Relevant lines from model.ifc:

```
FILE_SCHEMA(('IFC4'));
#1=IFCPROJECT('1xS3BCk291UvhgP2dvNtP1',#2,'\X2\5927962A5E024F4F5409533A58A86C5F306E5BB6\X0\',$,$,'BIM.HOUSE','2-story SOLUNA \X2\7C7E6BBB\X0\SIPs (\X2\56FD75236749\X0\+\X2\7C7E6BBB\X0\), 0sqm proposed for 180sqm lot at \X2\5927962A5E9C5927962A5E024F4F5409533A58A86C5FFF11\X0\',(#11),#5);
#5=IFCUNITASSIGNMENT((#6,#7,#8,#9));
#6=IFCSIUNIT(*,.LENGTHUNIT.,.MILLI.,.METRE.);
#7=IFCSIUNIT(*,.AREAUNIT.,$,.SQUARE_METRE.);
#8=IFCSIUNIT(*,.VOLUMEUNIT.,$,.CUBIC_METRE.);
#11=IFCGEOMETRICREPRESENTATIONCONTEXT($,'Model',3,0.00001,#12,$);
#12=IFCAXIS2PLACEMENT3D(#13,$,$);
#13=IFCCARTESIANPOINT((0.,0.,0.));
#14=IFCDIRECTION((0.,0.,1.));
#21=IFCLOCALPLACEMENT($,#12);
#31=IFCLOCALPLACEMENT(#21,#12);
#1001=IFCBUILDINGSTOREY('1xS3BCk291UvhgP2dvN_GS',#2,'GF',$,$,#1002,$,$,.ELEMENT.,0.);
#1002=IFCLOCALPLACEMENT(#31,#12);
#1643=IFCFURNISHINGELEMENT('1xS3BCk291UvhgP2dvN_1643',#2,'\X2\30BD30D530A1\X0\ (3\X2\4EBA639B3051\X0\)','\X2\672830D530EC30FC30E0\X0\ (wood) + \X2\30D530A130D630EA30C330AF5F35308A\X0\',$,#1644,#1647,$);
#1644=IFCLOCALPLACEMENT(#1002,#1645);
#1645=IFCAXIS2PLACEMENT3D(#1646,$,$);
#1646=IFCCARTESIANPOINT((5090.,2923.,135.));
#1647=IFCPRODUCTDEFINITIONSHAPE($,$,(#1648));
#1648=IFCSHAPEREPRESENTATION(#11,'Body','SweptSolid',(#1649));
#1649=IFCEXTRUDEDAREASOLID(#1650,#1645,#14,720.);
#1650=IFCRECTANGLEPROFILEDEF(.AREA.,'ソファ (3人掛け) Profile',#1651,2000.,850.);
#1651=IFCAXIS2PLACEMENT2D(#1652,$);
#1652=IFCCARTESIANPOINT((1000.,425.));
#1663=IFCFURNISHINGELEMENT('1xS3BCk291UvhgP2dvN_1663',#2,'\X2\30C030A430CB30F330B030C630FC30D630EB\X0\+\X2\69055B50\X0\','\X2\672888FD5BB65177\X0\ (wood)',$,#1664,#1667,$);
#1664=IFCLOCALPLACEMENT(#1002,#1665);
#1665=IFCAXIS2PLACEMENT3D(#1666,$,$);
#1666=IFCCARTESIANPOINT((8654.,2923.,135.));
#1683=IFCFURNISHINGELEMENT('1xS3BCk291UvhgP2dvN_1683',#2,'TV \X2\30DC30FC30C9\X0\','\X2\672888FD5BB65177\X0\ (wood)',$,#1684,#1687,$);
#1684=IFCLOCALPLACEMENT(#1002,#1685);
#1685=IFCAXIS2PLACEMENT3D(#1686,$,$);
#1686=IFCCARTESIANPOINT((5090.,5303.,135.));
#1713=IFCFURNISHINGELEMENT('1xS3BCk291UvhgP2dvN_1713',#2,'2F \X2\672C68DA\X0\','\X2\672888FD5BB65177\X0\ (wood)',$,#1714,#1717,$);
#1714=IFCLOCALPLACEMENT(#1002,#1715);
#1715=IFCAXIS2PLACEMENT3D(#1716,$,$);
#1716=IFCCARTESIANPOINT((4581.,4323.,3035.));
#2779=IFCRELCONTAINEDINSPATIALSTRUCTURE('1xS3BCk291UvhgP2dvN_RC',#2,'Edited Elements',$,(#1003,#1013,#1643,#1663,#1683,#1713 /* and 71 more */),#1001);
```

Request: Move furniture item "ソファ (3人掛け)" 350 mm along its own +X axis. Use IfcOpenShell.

```python
import ifcopenshell
import ifcopenshell.api.geometry
import ifcopenshell.util.placement

model = ifcopenshell.open("model.ifc")

item = model.by_guid("1xS3BCk291UvhgP2dvN_1643")
matrix = ifcopenshell.util.placement.get_local_placement(item.ObjectPlacement)
matrix[:3, 3] += matrix[:3, 0] * 350.0
ifcopenshell.api.geometry.edit_object_placement(model, product=item, matrix=matrix, is_si=False)

print(ifcopenshell.util.placement.get_local_placement(item.ObjectPlacement).round(3) + 0.0)

model.write("model-out.ifc")
```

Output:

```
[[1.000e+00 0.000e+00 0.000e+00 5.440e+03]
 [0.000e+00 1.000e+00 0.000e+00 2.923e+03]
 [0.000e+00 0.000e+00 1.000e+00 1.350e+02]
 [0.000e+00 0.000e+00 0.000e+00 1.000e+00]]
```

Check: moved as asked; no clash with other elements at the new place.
